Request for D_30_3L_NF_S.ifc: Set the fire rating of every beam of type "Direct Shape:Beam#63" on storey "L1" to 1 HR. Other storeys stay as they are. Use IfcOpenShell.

First a look at what the model holds.

```python
import ifcopenshell
import ifcopenshell.util.element

model = ifcopenshell.open("D_30_3L_NF_S.ifc")
print(model.schema)
storey = next(s for s in model.by_type("IfcBuildingStorey") if s.Name == "L1")
beams = [e for e in ifcopenshell.util.element.get_decomposition(storey) if e.is_a("IfcBeam")]
seen = {}
for e in beams:
    element_type = ifcopenshell.util.element.get_type(e)
    key = (element_type.Name if element_type != e and element_type else None, ifcopenshell.util.element.get_pset(e, "Pset_BeamCommon", "FireRating"))
    seen[key] = seen.get(key, 0) + 1
for (name, value), count in sorted(seen.items(), key=str):
    print(count, "x", name, "|", value)
```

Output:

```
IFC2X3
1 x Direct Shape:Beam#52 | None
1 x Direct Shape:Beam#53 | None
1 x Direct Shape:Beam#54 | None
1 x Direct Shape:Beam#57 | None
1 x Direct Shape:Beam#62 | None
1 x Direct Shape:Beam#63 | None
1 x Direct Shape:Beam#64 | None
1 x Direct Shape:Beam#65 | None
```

```python
import ifcopenshell
import ifcopenshell.api.pset
import ifcopenshell.util.element

model = ifcopenshell.open("D_30_3L_NF_S.ifc")

storey = next(s for s in model.by_type("IfcBuildingStorey") if s.Name == "L1")
beams = [e for e in ifcopenshell.util.element.get_decomposition(storey) if e.is_a("IfcBeam")]

count = 0
for e in beams:
    element_type = ifcopenshell.util.element.get_type(e)
    if element_type in (None, e) or element_type.Name != "Direct Shape:Beam#63":
        continue
    # add_pset returns the element's existing set when there is one.
    pset = ifcopenshell.api.pset.add_pset(model, product=e, name="Pset_BeamCommon")
    ifcopenshell.api.pset.edit_pset(model, pset=pset, properties={"FireRating": "1 HR"})
    count += 1

print(count, "beams updated")

model.write("D_30_3L_NF_S_edited.ifc")
```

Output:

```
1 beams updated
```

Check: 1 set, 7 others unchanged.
